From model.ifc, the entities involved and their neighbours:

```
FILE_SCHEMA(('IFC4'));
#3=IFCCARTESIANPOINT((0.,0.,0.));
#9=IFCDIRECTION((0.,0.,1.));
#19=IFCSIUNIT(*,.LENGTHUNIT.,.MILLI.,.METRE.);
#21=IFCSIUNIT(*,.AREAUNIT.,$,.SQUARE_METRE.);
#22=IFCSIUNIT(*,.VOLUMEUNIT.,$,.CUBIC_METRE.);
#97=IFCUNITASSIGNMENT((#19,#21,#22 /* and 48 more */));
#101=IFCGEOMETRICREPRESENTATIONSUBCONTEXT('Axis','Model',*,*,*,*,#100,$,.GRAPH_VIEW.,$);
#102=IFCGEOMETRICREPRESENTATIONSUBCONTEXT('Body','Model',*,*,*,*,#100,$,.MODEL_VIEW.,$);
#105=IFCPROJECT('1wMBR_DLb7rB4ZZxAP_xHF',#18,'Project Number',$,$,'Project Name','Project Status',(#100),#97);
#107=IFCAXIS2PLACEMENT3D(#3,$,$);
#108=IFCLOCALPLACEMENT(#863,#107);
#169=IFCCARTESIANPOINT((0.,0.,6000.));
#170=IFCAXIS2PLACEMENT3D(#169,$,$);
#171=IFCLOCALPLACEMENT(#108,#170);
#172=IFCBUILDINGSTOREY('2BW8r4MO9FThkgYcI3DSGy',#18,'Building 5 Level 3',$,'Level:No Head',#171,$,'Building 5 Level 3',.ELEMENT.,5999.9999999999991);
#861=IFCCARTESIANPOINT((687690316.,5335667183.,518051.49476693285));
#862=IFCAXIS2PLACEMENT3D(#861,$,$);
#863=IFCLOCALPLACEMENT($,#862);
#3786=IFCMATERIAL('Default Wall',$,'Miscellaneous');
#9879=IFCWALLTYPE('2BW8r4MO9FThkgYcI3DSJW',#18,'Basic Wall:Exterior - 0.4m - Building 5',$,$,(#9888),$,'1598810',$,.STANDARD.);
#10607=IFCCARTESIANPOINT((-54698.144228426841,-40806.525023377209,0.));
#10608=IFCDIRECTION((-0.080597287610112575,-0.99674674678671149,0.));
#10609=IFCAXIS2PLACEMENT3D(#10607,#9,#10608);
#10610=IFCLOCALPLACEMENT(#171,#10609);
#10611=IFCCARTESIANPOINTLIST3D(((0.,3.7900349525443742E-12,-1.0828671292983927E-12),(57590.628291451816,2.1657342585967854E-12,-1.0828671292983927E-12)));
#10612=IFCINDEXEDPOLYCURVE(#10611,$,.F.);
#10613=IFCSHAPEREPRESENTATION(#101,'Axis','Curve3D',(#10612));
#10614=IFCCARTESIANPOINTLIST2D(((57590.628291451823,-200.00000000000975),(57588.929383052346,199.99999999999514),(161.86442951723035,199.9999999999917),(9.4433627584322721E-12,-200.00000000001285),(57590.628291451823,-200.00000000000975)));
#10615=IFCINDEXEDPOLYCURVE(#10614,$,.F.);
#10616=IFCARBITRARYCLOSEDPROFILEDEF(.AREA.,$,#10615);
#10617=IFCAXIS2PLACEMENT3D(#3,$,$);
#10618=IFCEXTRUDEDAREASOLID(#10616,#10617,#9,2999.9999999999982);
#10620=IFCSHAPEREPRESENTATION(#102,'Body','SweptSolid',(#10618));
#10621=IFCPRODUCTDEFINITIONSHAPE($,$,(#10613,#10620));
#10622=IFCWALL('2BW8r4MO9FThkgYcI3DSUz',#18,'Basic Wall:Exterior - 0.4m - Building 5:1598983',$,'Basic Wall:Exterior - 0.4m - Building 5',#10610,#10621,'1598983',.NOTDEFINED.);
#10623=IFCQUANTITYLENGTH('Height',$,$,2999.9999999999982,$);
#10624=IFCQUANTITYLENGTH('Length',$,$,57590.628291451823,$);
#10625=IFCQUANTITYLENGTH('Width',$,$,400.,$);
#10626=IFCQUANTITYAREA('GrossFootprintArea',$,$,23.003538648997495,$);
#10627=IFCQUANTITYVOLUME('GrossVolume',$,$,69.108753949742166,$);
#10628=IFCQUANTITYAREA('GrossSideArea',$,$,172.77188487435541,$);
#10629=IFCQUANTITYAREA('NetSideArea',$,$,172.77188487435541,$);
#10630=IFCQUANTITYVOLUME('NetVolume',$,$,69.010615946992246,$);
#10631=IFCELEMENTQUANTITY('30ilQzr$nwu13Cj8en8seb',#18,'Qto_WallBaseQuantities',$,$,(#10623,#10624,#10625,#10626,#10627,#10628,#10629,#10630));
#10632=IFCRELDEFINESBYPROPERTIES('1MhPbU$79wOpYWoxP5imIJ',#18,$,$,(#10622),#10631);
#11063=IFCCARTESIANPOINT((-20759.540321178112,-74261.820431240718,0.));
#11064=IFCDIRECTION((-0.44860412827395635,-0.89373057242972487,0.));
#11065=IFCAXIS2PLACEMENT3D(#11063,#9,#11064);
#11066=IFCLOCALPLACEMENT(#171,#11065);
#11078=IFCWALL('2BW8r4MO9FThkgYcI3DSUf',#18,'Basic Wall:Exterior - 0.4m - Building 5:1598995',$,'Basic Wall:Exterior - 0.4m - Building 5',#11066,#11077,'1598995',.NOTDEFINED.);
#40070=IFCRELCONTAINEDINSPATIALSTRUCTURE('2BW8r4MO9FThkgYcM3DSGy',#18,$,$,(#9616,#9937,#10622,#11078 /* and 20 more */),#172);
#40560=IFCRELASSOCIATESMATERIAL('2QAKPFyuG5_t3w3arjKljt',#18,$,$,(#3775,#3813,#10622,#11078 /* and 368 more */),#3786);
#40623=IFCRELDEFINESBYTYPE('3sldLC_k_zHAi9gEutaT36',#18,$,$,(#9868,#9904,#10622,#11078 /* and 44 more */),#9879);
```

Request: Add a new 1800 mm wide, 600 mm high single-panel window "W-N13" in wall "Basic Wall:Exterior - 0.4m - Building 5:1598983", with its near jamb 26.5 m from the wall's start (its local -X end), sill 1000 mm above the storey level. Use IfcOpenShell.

```python
import numpy as np
import ifcopenshell
import ifcopenshell.api.feature
import ifcopenshell.api.geometry
import ifcopenshell.api.pset
import ifcopenshell.api.root
import ifcopenshell.api.spatial
import ifcopenshell.geom
import ifcopenshell.util.element
import ifcopenshell.util.placement
import ifcopenshell.util.representation
import ifcopenshell.util.shape
import ifcopenshell.util.unit

model = ifcopenshell.open("model.ifc")
unit_scale = ifcopenshell.util.unit.calculate_unit_scale(model)
area_scale = ifcopenshell.util.unit.calculate_unit_scale(model, "AREAUNIT")
volume_scale = ifcopenshell.util.unit.calculate_unit_scale(model, "VOLUMEUNIT")
settings = ifcopenshell.geom.settings()


def volume(element):
    """Net volume in cubic metres, openings subtracted."""
    shape = ifcopenshell.geom.create_shape(settings, element)
    return ifcopenshell.util.shape.get_volume(shape.geometry)


wall = model.by_guid("2BW8r4MO9FThkgYcI3DSUz")
storey = ifcopenshell.util.element.get_container(wall, ifc_class="IfcBuildingStorey")
context = ifcopenshell.util.representation.get_context(model, "Model", "Body", "MODEL_VIEW")
before = volume(wall)

width, height, from_end, sill = 1.8, 0.6, 26.5, 1  # metres

# The wall runs along its own X axis, and the end named is its -X end.
wall_shape = ifcopenshell.geom.create_shape(settings, wall)
x, y, z = ifcopenshell.util.shape.get_vertices(wall_shape.geometry).T
start = x.min() + from_end
face, thickness = float(y.min()), float(y.max() - y.min())
wall_matrix = ifcopenshell.util.placement.get_local_placement(wall.ObjectPlacement)
level = ifcopenshell.util.placement.get_local_placement(storey.ObjectPlacement)[2, 3]


def in_wall(x, y):
    """Placement at x, y metres in the wall's axes, at sill height."""
    matrix = wall_matrix.copy()
    matrix[:, 3] = wall_matrix @ np.array([x / unit_scale, y / unit_scale, 0.0, 1.0])
    matrix[2, 3] = level + sill / unit_scale
    return matrix


# Opening: a box that overshoots both wall faces by 50 mm.
opening = ifcopenshell.api.root.create_entity(model, ifc_class="IfcOpeningElement", predefined_type="OPENING")
box = ifcopenshell.api.geometry.add_wall_representation(
    model, context=context, length=width, height=height, thickness=thickness + 0.1
)
ifcopenshell.api.geometry.assign_representation(model, product=opening, representation=box)
ifcopenshell.api.geometry.edit_object_placement(model, product=opening, matrix=in_wall(start, face - 0.05), is_si=False)
ifcopenshell.api.feature.add_feature(model, feature=opening, element=wall)

window = ifcopenshell.api.root.create_entity(model, ifc_class="IfcWindow", name="W-N13", predefined_type="WINDOW")
window.OverallWidth, window.OverallHeight = width / unit_scale, height / unit_scale
window.PartitioningType = "SINGLE_PANEL"
body = ifcopenshell.api.geometry.add_window_representation(
    model,
    context=context,
    overall_width=window.OverallWidth,
    overall_height=window.OverallHeight,
    partition_type="SINGLE_PANEL",
)
ifcopenshell.api.geometry.assign_representation(model, product=window, representation=body)
ifcopenshell.api.spatial.assign_container(model, products=[window], relating_structure=storey)
ifcopenshell.api.feature.add_filling(model, opening=opening, element=window)

# Centre the window in the wall's thickness.
ifcopenshell.api.geometry.edit_object_placement(model, product=window, matrix=in_wall(start, face), is_si=False)
window_shape = ifcopenshell.geom.create_shape(settings, window)
depth = ifcopenshell.util.shape.get_vertices(window_shape.geometry)[:, 1]
offset = face + thickness / 2 - (depth.min() + depth.max()) / 2
ifcopenshell.api.geometry.edit_object_placement(model, product=window, matrix=in_wall(start, offset), is_si=False)

after = volume(wall)

# Update the wall's stored quantities.
qto = model.by_id(ifcopenshell.util.element.get_pset(wall, "Qto_WallBaseQuantities", should_inherit=False)["id"])
ifcopenshell.api.pset.edit_qto(model, qto=qto, properties={
    "NetSideArea": after / thickness / area_scale,
    "NetVolume": after / volume_scale,
})

print(f"wall volume {before:.3f} -> {after:.3f} m3")

model.write("model_updated.ifc")
```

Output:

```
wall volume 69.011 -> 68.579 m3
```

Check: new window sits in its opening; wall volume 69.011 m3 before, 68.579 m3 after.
